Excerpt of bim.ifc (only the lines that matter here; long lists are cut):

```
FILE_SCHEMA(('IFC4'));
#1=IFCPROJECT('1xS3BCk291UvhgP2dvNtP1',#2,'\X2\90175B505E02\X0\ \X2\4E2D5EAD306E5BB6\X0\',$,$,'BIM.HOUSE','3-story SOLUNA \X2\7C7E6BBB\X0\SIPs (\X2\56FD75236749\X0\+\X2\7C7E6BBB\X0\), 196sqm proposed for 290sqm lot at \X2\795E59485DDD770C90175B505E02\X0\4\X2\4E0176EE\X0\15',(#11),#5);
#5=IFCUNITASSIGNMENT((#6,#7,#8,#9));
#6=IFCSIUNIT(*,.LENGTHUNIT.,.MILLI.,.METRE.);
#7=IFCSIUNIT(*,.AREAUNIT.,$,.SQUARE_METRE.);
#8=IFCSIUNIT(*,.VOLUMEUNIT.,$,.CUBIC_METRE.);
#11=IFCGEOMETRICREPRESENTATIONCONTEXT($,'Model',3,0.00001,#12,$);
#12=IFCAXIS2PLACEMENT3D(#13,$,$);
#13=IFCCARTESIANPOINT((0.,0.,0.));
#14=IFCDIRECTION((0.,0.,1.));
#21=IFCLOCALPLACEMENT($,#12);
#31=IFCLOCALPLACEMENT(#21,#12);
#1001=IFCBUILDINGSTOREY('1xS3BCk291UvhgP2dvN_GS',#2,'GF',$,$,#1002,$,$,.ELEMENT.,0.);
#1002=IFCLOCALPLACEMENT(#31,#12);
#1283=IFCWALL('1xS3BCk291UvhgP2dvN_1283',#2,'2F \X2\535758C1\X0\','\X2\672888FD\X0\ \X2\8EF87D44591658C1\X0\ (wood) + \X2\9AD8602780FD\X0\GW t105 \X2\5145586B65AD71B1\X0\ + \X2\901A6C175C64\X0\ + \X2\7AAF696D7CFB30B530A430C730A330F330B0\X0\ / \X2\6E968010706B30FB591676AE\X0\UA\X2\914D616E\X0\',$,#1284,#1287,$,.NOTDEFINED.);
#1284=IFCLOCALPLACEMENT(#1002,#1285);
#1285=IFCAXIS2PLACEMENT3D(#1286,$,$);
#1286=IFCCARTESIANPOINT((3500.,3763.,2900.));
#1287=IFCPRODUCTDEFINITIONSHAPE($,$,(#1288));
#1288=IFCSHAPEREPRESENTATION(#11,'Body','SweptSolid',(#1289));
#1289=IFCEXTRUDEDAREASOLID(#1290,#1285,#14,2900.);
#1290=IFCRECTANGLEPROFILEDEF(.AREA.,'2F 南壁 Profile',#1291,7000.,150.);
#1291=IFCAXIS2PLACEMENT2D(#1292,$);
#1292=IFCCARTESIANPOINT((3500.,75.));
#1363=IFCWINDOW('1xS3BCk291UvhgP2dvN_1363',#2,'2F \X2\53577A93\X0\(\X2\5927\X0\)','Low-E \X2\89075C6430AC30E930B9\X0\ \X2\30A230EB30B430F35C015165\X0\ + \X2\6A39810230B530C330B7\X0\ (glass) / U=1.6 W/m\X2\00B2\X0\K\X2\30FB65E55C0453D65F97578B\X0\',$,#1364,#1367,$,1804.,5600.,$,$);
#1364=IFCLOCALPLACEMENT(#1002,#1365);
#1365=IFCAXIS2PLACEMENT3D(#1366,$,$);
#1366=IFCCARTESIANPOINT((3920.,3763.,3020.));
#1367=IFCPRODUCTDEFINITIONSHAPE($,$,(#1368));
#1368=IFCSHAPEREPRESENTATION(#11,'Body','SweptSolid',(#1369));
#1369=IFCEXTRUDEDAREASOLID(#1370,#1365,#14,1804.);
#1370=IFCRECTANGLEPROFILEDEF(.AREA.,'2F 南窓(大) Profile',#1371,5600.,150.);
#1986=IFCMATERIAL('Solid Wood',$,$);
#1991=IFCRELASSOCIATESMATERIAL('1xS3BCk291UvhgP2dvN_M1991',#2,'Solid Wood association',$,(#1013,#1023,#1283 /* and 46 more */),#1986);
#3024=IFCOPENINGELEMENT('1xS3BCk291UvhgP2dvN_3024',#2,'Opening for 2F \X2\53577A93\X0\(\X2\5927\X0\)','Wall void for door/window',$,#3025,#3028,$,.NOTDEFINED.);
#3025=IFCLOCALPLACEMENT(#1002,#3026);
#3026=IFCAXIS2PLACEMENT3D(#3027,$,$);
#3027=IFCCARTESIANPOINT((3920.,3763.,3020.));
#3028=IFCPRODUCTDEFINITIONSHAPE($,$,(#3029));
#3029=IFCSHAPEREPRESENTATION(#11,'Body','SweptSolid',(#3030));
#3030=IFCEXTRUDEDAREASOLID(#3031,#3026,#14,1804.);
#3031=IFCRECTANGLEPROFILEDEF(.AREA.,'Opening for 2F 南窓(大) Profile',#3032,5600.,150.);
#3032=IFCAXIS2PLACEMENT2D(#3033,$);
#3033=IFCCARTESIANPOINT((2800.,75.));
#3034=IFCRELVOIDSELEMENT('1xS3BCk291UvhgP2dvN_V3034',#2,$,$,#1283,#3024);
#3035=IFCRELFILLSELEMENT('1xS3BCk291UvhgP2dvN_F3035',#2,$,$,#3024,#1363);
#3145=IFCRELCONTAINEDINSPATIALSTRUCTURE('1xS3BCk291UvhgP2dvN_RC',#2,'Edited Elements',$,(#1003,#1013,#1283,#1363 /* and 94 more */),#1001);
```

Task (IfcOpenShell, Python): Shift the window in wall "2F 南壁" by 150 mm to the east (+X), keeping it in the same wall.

```python
import ifcopenshell
import ifcopenshell.api.geometry
import ifcopenshell.util.placement

model = ifcopenshell.open("bim.ifc")

window = model.by_id(1363)
opening = window.FillsVoids[0].RelatingOpeningElement
wall = opening.VoidsElements[0].RelatingBuildingElement

wall_matrix = ifcopenshell.util.placement.get_local_placement(wall.ObjectPlacement)
shift = wall_matrix[:3, 0] * 150.0
before = ifcopenshell.util.placement.get_local_placement(window.ObjectPlacement)[:3, 3].copy()

# The window is not placed relative to its opening, so move both.
for product in (opening, window):
    matrix = ifcopenshell.util.placement.get_local_placement(product.ObjectPlacement)
    matrix[:3, 3] += shift
    ifcopenshell.api.geometry.edit_object_placement(model, product=product, matrix=matrix, is_si=False)

after = ifcopenshell.util.placement.get_local_placement(window.ObjectPlacement)[:3, 3]
print("window moved by", (after - before).round(3) + 0.0)

model.write("bim_updated.ifc")
```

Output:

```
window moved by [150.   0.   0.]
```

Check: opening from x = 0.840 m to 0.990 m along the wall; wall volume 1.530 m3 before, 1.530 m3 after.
